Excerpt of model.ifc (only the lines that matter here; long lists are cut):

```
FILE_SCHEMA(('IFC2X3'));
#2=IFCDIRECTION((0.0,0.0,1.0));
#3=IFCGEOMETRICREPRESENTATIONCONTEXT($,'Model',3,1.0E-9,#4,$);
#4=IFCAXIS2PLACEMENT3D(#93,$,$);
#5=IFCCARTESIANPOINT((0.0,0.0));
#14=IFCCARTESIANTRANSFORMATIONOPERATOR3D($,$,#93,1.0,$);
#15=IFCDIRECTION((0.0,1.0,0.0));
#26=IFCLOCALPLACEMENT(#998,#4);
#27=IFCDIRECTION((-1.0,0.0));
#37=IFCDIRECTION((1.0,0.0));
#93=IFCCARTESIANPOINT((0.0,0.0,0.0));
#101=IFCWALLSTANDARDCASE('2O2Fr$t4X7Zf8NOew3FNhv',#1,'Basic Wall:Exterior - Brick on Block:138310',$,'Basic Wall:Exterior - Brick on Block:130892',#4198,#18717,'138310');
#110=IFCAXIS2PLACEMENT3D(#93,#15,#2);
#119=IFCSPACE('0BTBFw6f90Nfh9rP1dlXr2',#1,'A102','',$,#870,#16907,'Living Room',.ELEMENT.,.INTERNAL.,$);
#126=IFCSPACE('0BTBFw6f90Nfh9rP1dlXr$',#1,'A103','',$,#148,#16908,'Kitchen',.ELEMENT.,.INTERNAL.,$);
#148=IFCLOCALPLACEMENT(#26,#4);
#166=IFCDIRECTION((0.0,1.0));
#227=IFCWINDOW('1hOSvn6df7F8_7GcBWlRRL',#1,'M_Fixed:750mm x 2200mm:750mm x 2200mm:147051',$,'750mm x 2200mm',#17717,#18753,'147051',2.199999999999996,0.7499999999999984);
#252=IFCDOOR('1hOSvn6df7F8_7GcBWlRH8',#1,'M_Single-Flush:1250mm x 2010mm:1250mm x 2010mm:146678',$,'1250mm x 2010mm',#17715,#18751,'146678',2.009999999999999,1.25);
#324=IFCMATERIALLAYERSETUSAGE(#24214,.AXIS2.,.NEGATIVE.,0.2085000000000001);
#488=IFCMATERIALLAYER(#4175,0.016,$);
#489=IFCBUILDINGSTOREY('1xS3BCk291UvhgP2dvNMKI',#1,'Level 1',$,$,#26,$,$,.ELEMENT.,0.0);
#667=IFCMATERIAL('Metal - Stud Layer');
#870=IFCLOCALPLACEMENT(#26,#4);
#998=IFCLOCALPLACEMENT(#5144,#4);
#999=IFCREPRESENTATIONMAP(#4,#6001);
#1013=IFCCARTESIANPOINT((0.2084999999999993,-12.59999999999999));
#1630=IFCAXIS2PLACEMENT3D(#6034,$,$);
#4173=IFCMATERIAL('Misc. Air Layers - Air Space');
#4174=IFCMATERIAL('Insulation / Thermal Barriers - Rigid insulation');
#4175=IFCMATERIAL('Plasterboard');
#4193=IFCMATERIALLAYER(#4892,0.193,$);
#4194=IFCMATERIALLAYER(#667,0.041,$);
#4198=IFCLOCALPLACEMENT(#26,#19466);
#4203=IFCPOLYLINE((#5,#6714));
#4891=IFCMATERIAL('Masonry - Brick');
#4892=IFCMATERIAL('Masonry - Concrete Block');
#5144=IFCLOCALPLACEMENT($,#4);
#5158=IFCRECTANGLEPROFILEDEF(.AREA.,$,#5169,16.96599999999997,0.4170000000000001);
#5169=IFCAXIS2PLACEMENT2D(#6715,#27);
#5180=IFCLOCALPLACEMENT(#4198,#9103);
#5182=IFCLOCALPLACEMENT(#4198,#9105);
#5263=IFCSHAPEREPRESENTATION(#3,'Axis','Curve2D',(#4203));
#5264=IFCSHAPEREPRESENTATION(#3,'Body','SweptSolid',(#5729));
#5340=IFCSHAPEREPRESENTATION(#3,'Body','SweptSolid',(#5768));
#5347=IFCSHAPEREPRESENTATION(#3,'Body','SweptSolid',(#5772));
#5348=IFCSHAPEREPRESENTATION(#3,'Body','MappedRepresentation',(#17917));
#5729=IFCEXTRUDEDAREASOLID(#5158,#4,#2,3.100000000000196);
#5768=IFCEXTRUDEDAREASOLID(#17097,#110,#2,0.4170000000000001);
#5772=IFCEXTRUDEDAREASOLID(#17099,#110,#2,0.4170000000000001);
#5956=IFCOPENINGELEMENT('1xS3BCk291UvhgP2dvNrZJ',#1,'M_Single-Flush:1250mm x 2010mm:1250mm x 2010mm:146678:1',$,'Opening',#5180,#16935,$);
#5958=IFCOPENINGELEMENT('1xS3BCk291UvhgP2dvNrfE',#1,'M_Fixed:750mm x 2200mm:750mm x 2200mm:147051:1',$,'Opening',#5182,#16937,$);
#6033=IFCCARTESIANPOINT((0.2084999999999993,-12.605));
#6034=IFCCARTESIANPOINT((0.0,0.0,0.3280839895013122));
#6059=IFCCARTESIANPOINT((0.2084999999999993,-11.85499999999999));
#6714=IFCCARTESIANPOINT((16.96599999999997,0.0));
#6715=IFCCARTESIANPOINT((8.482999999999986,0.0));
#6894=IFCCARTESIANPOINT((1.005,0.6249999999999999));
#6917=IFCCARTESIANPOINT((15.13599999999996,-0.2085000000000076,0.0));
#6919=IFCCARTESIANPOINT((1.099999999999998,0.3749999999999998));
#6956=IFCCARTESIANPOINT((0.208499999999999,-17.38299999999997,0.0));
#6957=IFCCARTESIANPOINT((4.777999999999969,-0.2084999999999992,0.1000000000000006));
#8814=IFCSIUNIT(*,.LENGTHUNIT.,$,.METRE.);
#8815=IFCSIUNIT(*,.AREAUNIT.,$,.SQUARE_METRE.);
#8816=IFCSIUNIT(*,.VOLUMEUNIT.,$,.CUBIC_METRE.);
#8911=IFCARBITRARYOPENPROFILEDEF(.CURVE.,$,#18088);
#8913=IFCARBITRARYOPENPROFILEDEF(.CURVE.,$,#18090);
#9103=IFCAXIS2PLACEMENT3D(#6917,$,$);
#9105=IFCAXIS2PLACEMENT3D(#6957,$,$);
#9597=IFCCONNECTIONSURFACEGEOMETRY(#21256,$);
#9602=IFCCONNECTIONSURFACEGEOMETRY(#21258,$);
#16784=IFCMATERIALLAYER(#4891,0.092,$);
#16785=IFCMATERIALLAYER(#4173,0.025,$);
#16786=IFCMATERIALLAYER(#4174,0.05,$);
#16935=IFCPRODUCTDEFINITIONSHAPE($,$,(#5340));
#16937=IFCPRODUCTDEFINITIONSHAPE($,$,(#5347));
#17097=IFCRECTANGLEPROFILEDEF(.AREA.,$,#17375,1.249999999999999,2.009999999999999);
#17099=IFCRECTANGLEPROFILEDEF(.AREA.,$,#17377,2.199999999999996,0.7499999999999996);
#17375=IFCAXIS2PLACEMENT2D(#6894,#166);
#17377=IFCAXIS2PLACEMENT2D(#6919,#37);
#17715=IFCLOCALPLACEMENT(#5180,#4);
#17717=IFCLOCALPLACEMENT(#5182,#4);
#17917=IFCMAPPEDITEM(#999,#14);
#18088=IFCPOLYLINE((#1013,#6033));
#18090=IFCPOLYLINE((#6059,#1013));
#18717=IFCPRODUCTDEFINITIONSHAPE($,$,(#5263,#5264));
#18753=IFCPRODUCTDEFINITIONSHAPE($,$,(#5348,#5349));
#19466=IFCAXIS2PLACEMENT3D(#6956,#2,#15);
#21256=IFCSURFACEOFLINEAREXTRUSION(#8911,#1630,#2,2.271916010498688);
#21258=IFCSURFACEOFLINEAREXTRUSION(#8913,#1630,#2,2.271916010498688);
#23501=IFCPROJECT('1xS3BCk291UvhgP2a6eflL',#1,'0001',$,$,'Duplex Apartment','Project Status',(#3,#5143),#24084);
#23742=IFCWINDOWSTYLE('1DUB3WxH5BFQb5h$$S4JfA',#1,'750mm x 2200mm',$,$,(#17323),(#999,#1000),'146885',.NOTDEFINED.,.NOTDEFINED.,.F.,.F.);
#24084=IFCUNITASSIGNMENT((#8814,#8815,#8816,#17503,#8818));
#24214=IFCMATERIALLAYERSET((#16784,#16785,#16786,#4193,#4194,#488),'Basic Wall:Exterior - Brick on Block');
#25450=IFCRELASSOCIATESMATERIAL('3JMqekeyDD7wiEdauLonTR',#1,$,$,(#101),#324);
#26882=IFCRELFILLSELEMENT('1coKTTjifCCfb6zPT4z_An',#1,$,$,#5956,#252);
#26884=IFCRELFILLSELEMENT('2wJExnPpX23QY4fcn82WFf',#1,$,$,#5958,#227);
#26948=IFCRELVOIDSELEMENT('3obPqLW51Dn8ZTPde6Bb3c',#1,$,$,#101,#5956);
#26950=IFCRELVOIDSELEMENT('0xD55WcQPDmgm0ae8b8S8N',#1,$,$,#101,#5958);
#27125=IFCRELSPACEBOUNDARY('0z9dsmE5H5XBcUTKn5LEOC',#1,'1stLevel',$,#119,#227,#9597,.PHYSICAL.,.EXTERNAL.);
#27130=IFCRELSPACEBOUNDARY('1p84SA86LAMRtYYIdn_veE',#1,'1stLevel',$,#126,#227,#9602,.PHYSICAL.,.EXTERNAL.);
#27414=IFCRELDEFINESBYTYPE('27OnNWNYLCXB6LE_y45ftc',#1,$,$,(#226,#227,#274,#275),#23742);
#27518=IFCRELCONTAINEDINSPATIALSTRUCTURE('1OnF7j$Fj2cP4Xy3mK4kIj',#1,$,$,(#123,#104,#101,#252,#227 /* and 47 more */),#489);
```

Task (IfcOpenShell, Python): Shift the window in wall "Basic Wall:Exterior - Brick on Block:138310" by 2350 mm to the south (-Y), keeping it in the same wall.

```python
import numpy as np
import ifcopenshell
import ifcopenshell.api.geometry
import ifcopenshell.util.placement
import ifcopenshell.util.unit

model = ifcopenshell.open("model.ifc")
unit_scale = ifcopenshell.util.unit.calculate_unit_scale(model)

window = model.by_id(227)
opening = window.FillsVoids[0].RelatingOpeningElement
wall = opening.VoidsElements[0].RelatingBuildingElement

wall_matrix = ifcopenshell.util.placement.get_local_placement(wall.ObjectPlacement)
shift = wall_matrix[:3, 0] * -2.35 / unit_scale
before = ifcopenshell.util.placement.get_local_placement(window.ObjectPlacement)[:3, 3].copy()

# The window is placed relative to its opening, so it follows when the opening moves.
matrix = ifcopenshell.util.placement.get_local_placement(opening.ObjectPlacement)
matrix[:3, 3] += shift
ifcopenshell.api.geometry.edit_object_placement(
    model, product=opening, matrix=matrix, is_si=False, should_transform_children=True
)

# Space boundary surfaces are stored in each space's coordinates; move them too.
for rel in window.ProvidesBoundaries:
    if not rel.ConnectionGeometry:
        continue
    surface = rel.ConnectionGeometry.SurfaceOnRelatingElement
    space_matrix = ifcopenshell.util.placement.get_local_placement(rel.RelatingSpace.ObjectPlacement)
    point = np.array(surface.Position.Location.Coordinates) + space_matrix[:3, :3].T @ shift
    surface.Position = model.createIfcAxis2Placement3D(
        model.createIfcCartesianPoint(point.tolist()), surface.Position.Axis, surface.Position.RefDirection
    )

after = ifcopenshell.util.placement.get_local_placement(window.ObjectPlacement)[:3, 3]
print("window moved by", (after - before).round(3) + 0.0)

model.write("model_rev.ifc")
```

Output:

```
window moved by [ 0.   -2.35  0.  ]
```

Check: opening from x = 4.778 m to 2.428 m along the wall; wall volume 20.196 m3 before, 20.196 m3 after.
